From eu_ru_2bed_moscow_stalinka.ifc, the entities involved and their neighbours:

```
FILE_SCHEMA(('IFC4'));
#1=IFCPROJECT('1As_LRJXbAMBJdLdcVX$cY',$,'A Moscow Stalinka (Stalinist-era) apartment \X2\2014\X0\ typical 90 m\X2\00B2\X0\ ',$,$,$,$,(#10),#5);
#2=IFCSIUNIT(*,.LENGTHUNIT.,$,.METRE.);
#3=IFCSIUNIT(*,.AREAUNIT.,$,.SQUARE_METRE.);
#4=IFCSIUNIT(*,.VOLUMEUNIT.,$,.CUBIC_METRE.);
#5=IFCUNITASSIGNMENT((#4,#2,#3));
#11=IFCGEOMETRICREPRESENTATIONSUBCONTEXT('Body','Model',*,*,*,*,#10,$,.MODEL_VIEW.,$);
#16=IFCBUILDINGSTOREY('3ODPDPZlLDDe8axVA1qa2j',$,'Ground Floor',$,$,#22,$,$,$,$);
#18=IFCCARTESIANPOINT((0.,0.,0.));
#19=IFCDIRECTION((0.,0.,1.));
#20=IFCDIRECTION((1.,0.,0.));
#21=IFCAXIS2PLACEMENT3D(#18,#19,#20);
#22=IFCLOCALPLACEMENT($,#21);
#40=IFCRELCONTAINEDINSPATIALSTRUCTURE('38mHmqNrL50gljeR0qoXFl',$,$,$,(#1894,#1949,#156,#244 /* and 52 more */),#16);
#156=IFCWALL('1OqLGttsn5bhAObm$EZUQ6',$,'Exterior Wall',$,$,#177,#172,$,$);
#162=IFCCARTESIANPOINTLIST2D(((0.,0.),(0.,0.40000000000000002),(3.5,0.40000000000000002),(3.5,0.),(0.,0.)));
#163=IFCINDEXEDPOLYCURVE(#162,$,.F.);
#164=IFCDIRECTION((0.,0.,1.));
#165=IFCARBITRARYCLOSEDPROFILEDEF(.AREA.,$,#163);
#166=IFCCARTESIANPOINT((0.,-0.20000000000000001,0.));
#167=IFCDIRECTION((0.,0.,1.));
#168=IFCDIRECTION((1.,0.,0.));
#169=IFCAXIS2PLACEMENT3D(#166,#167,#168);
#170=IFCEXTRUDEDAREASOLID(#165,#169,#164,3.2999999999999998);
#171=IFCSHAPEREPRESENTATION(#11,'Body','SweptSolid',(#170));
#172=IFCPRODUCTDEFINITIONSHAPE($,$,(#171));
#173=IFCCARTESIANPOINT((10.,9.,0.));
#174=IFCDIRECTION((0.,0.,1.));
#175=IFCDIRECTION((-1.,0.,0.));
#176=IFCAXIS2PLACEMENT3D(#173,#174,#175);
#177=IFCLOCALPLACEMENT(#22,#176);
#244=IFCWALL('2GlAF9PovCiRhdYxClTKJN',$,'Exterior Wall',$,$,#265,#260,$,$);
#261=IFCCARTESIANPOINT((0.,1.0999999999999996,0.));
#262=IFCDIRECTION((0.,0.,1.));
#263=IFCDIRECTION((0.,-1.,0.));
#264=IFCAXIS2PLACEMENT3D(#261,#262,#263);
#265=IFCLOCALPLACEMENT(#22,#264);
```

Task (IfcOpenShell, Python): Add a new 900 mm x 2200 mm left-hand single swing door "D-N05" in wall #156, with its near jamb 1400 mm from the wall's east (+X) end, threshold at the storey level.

```python
import numpy as np
import ifcopenshell
import ifcopenshell.api.feature
import ifcopenshell.api.geometry
import ifcopenshell.api.root
import ifcopenshell.api.spatial
import ifcopenshell.geom
import ifcopenshell.util.element
import ifcopenshell.util.placement
import ifcopenshell.util.representation
import ifcopenshell.util.shape
import ifcopenshell.util.unit

model = ifcopenshell.open("eu_ru_2bed_moscow_stalinka.ifc")
unit_scale = ifcopenshell.util.unit.calculate_unit_scale(model)
settings = ifcopenshell.geom.settings()


def volume(element):
    """Net volume in cubic metres, openings subtracted."""
    shape = ifcopenshell.geom.create_shape(settings, element)
    return ifcopenshell.util.shape.get_volume(shape.geometry)


wall = model.by_id(156)
storey = ifcopenshell.util.element.get_container(wall, ifc_class="IfcBuildingStorey")
context = ifcopenshell.util.representation.get_context(model, "Model", "Body", "MODEL_VIEW")
before = volume(wall)

width, height, from_end, sill = 0.9, 2.2, 1.4, 0.0  # metres

# The wall runs along its own X axis, and the end named is its -X end.
wall_shape = ifcopenshell.geom.create_shape(settings, wall)
x, y, z = ifcopenshell.util.shape.get_vertices(wall_shape.geometry).T
start = x.min() + from_end
face, thickness = float(y.min()), float(y.max() - y.min())
wall_matrix = ifcopenshell.util.placement.get_local_placement(wall.ObjectPlacement)
level = ifcopenshell.util.placement.get_local_placement(storey.ObjectPlacement)[2, 3]


def in_wall(x, y):
    """Placement at x, y metres in the wall's axes, at sill height."""
    matrix = wall_matrix.copy()
    matrix[:, 3] = wall_matrix @ np.array([x / unit_scale, y / unit_scale, 0.0, 1.0])
    matrix[2, 3] = level + sill / unit_scale
    return matrix


# Opening: a box that overshoots both wall faces by 50 mm.
opening = ifcopenshell.api.root.create_entity(model, ifc_class="IfcOpeningElement", predefined_type="OPENING")
box = ifcopenshell.api.geometry.add_wall_representation(
    model, context=context, length=width, height=height, thickness=thickness + 0.1
)
ifcopenshell.api.geometry.assign_representation(model, product=opening, representation=box)
ifcopenshell.api.geometry.edit_object_placement(model, product=opening, matrix=in_wall(start, face - 0.05), is_si=False)
ifcopenshell.api.feature.add_feature(model, feature=opening, element=wall)

door = ifcopenshell.api.root.create_entity(model, ifc_class="IfcDoor", name="D-N05", predefined_type="DOOR")
door.OverallWidth, door.OverallHeight = width / unit_scale, height / unit_scale
door.OperationType = "SINGLE_SWING_LEFT"
body = ifcopenshell.api.geometry.add_door_representation(
    model,
    context=context,
    overall_width=door.OverallWidth,
    overall_height=door.OverallHeight,
    operation_type="SINGLE_SWING_LEFT",
    lining_properties={"LiningDepth": thickness / unit_scale, "ThresholdDepth": thickness / unit_scale},
)
ifcopenshell.api.geometry.assign_representation(model, product=door, representation=body)
ifcopenshell.api.spatial.assign_container(model, products=[door], relating_structure=storey)
ifcopenshell.api.feature.add_filling(model, opening=opening, element=door)

# The lining spans the wall, so the door starts at the wall face.
ifcopenshell.api.geometry.edit_object_placement(model, product=door, matrix=in_wall(start, face), is_si=False)

after = volume(wall)

print(f"wall volume {before:.3f} -> {after:.3f} m3")

model.write("eu_ru_2bed_moscow_stalinka_edited.ifc")
```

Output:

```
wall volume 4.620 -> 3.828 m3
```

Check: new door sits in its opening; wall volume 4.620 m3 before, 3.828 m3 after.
